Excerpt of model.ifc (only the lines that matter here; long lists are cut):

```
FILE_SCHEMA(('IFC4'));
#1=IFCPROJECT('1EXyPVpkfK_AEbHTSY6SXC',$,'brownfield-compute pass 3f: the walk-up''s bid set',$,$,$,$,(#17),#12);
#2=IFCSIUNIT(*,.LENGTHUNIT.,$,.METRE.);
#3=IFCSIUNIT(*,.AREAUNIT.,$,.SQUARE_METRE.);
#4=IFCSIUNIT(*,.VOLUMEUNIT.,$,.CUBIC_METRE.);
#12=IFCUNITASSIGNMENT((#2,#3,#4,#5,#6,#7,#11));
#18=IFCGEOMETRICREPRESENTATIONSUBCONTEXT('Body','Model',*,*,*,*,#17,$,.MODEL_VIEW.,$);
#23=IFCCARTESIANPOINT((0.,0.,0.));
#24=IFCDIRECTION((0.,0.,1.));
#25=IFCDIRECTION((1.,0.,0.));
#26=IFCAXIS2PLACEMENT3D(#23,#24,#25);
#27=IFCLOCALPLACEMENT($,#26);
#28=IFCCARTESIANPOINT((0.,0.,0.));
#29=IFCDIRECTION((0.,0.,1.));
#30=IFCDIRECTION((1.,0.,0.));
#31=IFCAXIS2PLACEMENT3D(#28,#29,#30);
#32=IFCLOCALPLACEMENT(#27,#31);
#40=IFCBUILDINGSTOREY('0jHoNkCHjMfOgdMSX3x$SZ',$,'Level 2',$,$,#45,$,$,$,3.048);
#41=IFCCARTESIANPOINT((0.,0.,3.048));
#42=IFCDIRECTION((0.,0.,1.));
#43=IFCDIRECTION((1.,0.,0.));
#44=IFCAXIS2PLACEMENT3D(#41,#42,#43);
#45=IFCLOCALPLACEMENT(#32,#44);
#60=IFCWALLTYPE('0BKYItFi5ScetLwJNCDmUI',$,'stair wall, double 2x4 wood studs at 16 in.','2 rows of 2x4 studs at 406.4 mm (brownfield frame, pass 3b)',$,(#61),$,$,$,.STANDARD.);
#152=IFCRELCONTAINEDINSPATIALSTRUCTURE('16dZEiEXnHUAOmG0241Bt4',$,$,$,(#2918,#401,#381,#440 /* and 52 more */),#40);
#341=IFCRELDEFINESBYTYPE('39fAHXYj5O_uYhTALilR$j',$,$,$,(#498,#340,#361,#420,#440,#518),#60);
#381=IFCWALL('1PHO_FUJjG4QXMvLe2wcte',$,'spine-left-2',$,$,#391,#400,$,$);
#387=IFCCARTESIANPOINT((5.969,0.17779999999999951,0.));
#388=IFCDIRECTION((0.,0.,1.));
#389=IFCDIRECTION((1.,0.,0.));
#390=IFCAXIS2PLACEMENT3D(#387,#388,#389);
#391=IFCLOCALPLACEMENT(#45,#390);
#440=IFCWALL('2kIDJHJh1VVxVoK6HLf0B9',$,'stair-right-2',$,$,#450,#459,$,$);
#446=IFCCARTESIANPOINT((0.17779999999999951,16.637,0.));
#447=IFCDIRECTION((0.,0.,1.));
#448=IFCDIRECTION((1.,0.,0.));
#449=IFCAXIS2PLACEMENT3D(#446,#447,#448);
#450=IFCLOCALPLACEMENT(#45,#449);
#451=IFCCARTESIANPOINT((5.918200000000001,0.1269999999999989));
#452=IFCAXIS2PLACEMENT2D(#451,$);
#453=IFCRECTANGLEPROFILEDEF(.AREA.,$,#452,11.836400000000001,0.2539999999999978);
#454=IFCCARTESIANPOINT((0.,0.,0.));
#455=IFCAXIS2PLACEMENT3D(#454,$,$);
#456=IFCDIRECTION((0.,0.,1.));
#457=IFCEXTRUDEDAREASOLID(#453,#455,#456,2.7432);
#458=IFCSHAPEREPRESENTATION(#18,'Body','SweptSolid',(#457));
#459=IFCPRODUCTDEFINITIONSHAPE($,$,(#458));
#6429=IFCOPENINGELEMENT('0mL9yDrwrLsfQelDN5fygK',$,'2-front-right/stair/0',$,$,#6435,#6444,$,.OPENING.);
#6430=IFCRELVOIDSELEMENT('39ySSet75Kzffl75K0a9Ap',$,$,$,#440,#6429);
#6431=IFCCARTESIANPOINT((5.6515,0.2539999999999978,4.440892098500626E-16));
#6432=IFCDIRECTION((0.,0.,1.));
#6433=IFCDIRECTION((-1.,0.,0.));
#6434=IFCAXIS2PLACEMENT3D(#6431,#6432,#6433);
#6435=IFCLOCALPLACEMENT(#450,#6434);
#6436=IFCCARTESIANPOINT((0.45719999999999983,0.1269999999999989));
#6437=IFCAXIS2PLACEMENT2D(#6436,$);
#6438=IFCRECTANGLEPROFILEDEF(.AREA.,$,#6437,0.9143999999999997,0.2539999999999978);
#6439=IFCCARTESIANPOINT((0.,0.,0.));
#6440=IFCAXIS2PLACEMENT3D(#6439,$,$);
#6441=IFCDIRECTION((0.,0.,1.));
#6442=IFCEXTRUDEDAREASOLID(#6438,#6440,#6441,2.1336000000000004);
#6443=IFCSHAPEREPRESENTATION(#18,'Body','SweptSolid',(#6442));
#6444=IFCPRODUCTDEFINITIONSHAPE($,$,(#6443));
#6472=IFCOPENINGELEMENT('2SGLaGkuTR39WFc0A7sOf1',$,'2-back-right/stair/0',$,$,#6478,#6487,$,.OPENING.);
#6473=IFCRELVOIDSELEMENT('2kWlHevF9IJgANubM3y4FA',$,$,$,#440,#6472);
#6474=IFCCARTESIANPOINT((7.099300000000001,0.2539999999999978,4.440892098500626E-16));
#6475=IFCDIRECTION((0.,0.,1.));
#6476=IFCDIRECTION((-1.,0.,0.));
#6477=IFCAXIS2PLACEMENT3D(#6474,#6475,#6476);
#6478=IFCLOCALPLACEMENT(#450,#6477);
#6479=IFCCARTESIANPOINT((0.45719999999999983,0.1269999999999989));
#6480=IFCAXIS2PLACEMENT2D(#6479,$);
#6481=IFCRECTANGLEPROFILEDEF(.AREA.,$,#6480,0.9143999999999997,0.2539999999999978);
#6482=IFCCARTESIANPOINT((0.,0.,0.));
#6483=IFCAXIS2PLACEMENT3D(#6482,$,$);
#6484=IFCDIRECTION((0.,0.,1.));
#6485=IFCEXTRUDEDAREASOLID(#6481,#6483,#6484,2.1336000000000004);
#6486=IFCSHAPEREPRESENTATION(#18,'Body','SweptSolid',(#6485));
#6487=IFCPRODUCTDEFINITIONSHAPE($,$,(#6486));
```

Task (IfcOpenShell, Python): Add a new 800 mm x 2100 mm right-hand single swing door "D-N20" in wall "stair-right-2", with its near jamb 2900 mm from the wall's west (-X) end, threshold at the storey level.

```python
import numpy as np
import ifcopenshell
import ifcopenshell.api.feature
import ifcopenshell.api.geometry
import ifcopenshell.api.root
import ifcopenshell.api.spatial
import ifcopenshell.geom
import ifcopenshell.util.element
import ifcopenshell.util.placement
import ifcopenshell.util.representation
import ifcopenshell.util.shape
import ifcopenshell.util.unit

model = ifcopenshell.open("model.ifc")
unit_scale = ifcopenshell.util.unit.calculate_unit_scale(model)
settings = ifcopenshell.geom.settings()


def volume(element):
    """Net volume in cubic metres, openings subtracted."""
    shape = ifcopenshell.geom.create_shape(settings, element)
    return ifcopenshell.util.shape.get_volume(shape.geometry)


wall = model.by_guid("2kIDJHJh1VVxVoK6HLf0B9")
storey = ifcopenshell.util.element.get_container(wall, ifc_class="IfcBuildingStorey")
context = ifcopenshell.util.representation.get_context(model, "Model", "Body", "MODEL_VIEW")
before = volume(wall)

width, height, from_end, sill = 0.8, 2.1, 2.9, 0.0  # metres

# The wall runs along its own X axis, and the end named is its -X end.
wall_shape = ifcopenshell.geom.create_shape(settings, wall)
x, y, z = ifcopenshell.util.shape.get_vertices(wall_shape.geometry).T
start = x.min() + from_end
face, thickness = float(y.min()), float(y.max() - y.min())
wall_matrix = ifcopenshell.util.placement.get_local_placement(wall.ObjectPlacement)
level = ifcopenshell.util.placement.get_local_placement(storey.ObjectPlacement)[2, 3]


def in_wall(x, y):
    """Placement at x, y metres in the wall's axes, at sill height."""
    matrix = wall_matrix.copy()
    matrix[:, 3] = wall_matrix @ np.array([x / unit_scale, y / unit_scale, 0.0, 1.0])
    matrix[2, 3] = level + sill / unit_scale
    return matrix


# Opening: a box that overshoots both wall faces by 50 mm.
opening = ifcopenshell.api.root.create_entity(model, ifc_class="IfcOpeningElement", predefined_type="OPENING")
box = ifcopenshell.api.geometry.add_wall_representation(
    model, context=context, length=width, height=height, thickness=thickness + 0.1
)
ifcopenshell.api.geometry.assign_representation(model, product=opening, representation=box)
ifcopenshell.api.geometry.edit_object_placement(model, product=opening, matrix=in_wall(start, face - 0.05), is_si=False)
ifcopenshell.api.feature.add_feature(model, feature=opening, element=wall)

door = ifcopenshell.api.root.create_entity(model, ifc_class="IfcDoor", name="D-N20", predefined_type="DOOR")
door.OverallWidth, door.OverallHeight = width / unit_scale, height / unit_scale
door.OperationType = "SINGLE_SWING_RIGHT"
body = ifcopenshell.api.geometry.add_door_representation(
    model,
    context=context,
    overall_width=door.OverallWidth,
    overall_height=door.OverallHeight,
    operation_type="SINGLE_SWING_RIGHT",
    lining_properties={"LiningDepth": thickness / unit_scale, "ThresholdDepth": thickness / unit_scale},
)
ifcopenshell.api.geometry.assign_representation(model, product=door, representation=body)
ifcopenshell.api.spatial.assign_container(model, products=[door], relating_structure=storey)
ifcopenshell.api.feature.add_filling(model, opening=opening, element=door)

# The lining spans the wall, so the door starts at the wall face.
ifcopenshell.api.geometry.edit_object_placement(model, product=door, matrix=in_wall(start, face), is_si=False)

after = volume(wall)

print(f"wall volume {before:.3f} -> {after:.3f} m3")

model.write("model_updated.ifc")
```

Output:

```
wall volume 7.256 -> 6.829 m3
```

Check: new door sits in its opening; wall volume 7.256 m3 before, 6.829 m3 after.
